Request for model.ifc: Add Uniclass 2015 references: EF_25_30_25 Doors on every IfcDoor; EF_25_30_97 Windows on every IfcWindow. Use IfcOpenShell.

First a look at what the model holds.

```python
import ifcopenshell

model = ifcopenshell.open("model.ifc")
print(model.schema)
print("classifications:", [c.Name for c in model.by_type("IfcClassification")])
for ifc_class in ("IfcDoor", "IfcRoof", "IfcStair", "IfcWall", "IfcWindow"):
    print(ifc_class, len(model.by_type(ifc_class)))
```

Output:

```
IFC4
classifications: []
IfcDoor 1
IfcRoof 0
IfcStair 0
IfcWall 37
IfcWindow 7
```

```python
import ifcopenshell
import ifcopenshell.api.classification

model = ifcopenshell.open("model.ifc")

system = ifcopenshell.api.classification.add_classification(model, classification="Uniclass 2015")

codes = {
    "IfcDoor": ("EF_25_30_25", "Doors"),
    "IfcWindow": ("EF_25_30_97", "Windows"),
}
for ifc_class, (code, name) in codes.items():
    products = model.by_type(ifc_class)
    ifcopenshell.api.classification.add_reference(
        model, products=products, classification=system, identification=code, name=name
    )
    print(code, len(products))

model.write("model_updated.ifc")
```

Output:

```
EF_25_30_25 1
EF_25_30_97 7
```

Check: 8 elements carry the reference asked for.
